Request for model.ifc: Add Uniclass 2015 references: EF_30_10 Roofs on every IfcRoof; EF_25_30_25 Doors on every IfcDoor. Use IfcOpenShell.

First a look at what the model holds.

```python
import ifcopenshell

model = ifcopenshell.open("model.ifc")
print(model.schema)
print("classifications:", [c.Name for c in model.by_type("IfcClassification")])
for ifc_class in ("IfcDoor", "IfcRoof", "IfcStair", "IfcWall", "IfcWindow"):
    print(ifc_class, len(model.by_type(ifc_class)))
```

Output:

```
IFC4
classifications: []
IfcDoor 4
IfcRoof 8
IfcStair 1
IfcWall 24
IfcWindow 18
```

```python
import ifcopenshell
import ifcopenshell.api.classification

model = ifcopenshell.open("model.ifc")

system = ifcopenshell.api.classification.add_classification(model, classification="Uniclass 2015")

codes = {
    "IfcRoof": ("EF_30_10", "Roofs"),
    "IfcDoor": ("EF_25_30_25", "Doors"),
}
for ifc_class, (code, name) in codes.items():
    products = model.by_type(ifc_class)
    ifcopenshell.api.classification.add_reference(
        model, products=products, classification=system, identification=code, name=name
    )
    print(code, len(products))

model.write("model-out.ifc")
```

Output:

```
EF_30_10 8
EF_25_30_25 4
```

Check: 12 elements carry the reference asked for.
